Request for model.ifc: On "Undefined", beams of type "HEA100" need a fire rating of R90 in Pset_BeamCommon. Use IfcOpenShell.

First a look at what the model holds.

```python
import ifcopenshell
import ifcopenshell.util.element

model = ifcopenshell.open("model.ifc")
print(model.schema)
storey = next(s for s in model.by_type("IfcBuildingStorey") if s.Name == "Undefined")
beams = [e for e in ifcopenshell.util.element.get_decomposition(storey) if e.is_a("IfcBeam")]
seen = {}
for e in beams:
    element_type = ifcopenshell.util.element.get_type(e)
    key = (element_type.Name if element_type != e and element_type else None, ifcopenshell.util.element.get_pset(e, "Pset_BeamCommon", "FireRating"))
    seen[key] = seen.get(key, 0) + 1
for (name, value), count in sorted(seen.items(), key=str):
    print(count, "x", name, "|", value)
```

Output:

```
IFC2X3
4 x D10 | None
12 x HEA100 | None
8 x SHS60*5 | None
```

```python
import ifcopenshell
import ifcopenshell.api.pset
import ifcopenshell.util.element

model = ifcopenshell.open("model.ifc")

storey = next(s for s in model.by_type("IfcBuildingStorey") if s.Name == "Undefined")
beams = [e for e in ifcopenshell.util.element.get_decomposition(storey) if e.is_a("IfcBeam")]

count = 0
for e in beams:
    element_type = ifcopenshell.util.element.get_type(e)
    if element_type in (None, e) or element_type.Name != "HEA100":
        continue
    # add_pset returns the element's existing set when there is one.
    pset = ifcopenshell.api.pset.add_pset(model, product=e, name="Pset_BeamCommon")
    ifcopenshell.api.pset.edit_pset(model, pset=pset, properties={"FireRating": "R90"})
    count += 1

print(count, "beams updated")

model.write("model_updated.ifc")
```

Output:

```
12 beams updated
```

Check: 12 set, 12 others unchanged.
